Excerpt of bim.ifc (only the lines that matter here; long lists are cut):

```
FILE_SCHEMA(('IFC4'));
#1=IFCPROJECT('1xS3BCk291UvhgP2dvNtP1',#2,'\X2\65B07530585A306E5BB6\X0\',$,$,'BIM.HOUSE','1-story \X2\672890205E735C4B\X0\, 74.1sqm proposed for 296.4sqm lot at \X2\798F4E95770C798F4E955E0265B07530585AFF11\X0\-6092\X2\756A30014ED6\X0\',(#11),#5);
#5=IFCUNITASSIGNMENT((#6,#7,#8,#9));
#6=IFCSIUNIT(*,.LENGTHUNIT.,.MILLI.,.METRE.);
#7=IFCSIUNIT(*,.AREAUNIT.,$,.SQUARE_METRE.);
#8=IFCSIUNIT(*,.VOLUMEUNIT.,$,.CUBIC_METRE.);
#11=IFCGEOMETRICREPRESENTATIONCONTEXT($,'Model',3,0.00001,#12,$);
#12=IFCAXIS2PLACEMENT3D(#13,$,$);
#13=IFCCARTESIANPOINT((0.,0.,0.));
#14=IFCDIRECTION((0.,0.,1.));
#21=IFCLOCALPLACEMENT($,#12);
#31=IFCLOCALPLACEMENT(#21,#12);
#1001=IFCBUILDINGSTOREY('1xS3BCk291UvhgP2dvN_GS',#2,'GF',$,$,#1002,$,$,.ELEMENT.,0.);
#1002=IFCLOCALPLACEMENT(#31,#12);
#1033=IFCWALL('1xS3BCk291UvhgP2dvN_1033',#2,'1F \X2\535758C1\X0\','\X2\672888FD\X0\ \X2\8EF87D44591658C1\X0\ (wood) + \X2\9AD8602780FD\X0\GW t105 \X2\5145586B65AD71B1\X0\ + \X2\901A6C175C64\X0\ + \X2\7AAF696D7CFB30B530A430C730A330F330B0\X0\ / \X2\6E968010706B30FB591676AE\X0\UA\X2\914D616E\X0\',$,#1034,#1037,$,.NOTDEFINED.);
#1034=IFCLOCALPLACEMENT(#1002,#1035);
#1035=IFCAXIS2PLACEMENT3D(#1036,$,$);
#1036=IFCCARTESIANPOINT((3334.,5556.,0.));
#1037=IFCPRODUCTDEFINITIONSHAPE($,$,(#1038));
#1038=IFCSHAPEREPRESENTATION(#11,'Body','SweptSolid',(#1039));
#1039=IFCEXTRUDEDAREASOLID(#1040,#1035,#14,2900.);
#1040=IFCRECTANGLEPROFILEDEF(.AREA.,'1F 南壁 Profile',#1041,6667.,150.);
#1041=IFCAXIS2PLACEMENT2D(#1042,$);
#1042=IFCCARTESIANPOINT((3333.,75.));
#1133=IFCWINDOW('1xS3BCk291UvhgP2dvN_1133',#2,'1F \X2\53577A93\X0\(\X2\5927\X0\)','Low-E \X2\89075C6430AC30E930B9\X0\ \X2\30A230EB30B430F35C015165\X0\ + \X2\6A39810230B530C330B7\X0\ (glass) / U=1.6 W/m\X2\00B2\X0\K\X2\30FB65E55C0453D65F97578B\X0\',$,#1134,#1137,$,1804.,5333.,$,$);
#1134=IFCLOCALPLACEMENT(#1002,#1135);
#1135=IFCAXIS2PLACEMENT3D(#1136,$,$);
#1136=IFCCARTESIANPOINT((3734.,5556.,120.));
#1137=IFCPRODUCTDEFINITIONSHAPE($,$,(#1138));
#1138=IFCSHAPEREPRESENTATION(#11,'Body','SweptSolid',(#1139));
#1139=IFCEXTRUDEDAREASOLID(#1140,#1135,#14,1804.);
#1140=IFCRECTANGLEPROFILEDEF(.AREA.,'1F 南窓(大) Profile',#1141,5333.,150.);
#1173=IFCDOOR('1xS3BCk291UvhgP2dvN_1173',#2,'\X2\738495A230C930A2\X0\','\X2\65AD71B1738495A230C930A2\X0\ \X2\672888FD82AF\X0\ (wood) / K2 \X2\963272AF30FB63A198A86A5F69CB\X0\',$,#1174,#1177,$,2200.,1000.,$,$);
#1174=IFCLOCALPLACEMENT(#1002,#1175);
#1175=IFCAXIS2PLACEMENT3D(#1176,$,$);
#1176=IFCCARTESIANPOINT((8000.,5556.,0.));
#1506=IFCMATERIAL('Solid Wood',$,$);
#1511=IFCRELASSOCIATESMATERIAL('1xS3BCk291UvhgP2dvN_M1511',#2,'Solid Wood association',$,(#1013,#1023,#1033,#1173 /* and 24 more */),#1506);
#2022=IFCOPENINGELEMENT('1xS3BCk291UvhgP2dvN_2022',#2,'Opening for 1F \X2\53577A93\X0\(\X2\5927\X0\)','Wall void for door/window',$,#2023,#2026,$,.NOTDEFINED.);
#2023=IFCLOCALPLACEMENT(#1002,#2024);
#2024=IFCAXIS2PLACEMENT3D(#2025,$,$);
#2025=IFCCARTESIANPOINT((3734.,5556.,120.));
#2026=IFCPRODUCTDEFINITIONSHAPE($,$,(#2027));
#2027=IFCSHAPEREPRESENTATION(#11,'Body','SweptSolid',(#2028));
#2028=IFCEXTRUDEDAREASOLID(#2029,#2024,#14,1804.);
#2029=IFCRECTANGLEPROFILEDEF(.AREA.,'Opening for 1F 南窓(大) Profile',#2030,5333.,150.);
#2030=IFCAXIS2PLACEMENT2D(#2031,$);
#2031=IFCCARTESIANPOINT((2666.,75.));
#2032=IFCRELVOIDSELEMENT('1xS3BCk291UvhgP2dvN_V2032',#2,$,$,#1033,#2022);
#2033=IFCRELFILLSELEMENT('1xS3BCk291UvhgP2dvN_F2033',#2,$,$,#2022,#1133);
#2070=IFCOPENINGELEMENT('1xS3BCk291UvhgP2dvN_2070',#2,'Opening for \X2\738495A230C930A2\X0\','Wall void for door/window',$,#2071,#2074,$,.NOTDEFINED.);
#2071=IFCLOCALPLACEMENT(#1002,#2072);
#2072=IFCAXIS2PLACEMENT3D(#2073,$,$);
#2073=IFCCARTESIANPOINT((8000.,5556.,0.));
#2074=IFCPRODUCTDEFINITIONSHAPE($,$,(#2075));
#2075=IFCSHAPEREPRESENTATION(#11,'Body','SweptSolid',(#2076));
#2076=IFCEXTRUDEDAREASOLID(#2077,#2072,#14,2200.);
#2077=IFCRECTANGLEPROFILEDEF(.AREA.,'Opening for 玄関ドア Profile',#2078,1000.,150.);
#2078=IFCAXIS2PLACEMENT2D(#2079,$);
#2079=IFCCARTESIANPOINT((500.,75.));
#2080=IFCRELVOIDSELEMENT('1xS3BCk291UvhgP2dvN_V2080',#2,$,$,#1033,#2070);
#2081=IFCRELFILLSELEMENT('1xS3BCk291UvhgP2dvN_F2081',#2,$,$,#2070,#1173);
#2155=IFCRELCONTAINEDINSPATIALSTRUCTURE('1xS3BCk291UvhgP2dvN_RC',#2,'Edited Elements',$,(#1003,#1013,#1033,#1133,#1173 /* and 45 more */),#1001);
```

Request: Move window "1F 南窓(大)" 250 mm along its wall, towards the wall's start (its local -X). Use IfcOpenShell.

```python
import ifcopenshell
import ifcopenshell.api.geometry
import ifcopenshell.util.placement
import ifcopenshell.util.unit

model = ifcopenshell.open("bim.ifc")
unit_scale = ifcopenshell.util.unit.calculate_unit_scale(model)

window = model.by_guid("1xS3BCk291UvhgP2dvN_1133")
opening = window.FillsVoids[0].RelatingOpeningElement
wall = opening.VoidsElements[0].RelatingBuildingElement

wall_matrix = ifcopenshell.util.placement.get_local_placement(wall.ObjectPlacement)
shift = wall_matrix[:3, 0] * -0.25 / unit_scale
before = ifcopenshell.util.placement.get_local_placement(window.ObjectPlacement)[:3, 3].copy()

# The window is not placed relative to its opening, so move both.
for product in (opening, window):
    matrix = ifcopenshell.util.placement.get_local_placement(product.ObjectPlacement)
    matrix[:3, 3] += shift
    ifcopenshell.api.geometry.edit_object_placement(model, product=product, matrix=matrix, is_si=False)

after = ifcopenshell.util.placement.get_local_placement(window.ObjectPlacement)[:3, 3]
print("window moved by", (after - before).round(3) + 0.0)

model.write("bim_edited.ifc")
```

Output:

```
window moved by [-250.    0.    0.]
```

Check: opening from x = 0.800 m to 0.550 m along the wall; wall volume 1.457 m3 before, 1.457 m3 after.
